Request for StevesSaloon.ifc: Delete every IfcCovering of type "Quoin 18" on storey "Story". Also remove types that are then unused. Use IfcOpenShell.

First a look at what the model holds.

```python
import ifcopenshell
import ifcopenshell.util.element

model = ifcopenshell.open("StevesSaloon.ifc")
print(model.schema)
storey = next(s for s in model.by_type("IfcBuildingStorey") if s.Name == "Story")
coverings = [e for e in ifcopenshell.util.element.get_decomposition(storey) if e.is_a("IfcCovering")]
seen = {}
for e in coverings:
    element_type = ifcopenshell.util.element.get_type(e)
    name = element_type.Name if element_type not in (None, e) else None
    seen[name] = seen.get(name, 0) + 1
for name, count in sorted(seen.items(), key=str):
    print(count, "x", name)
```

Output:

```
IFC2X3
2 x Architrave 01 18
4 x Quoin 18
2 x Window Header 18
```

```python
import ifcopenshell
import ifcopenshell.api.root
import ifcopenshell.util.element

model = ifcopenshell.open("StevesSaloon.ifc")

storey = next(s for s in model.by_type("IfcBuildingStorey") if s.Name == "Story")
coverings = [e for e in ifcopenshell.util.element.get_decomposition(storey) if e.is_a("IfcCovering")]
targets = [e for e in coverings if (t := ifcopenshell.util.element.get_type(e)) not in (None, e) and t.Name == "Quoin 18"]
types = {ifcopenshell.util.element.get_type(e) for e in targets} - {None, *targets}

for e in targets:
    ifcopenshell.api.root.remove_product(model, product=e)
print(len(targets), "removed")

unused = [t for t in types if not ifcopenshell.util.element.get_types(t)]
for t in unused:
    ifcopenshell.api.root.remove_product(model, product=t)
print(len(unused), "unused types removed")

model.write("StevesSaloon_updated.ifc")
```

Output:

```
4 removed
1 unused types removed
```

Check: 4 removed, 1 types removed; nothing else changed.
